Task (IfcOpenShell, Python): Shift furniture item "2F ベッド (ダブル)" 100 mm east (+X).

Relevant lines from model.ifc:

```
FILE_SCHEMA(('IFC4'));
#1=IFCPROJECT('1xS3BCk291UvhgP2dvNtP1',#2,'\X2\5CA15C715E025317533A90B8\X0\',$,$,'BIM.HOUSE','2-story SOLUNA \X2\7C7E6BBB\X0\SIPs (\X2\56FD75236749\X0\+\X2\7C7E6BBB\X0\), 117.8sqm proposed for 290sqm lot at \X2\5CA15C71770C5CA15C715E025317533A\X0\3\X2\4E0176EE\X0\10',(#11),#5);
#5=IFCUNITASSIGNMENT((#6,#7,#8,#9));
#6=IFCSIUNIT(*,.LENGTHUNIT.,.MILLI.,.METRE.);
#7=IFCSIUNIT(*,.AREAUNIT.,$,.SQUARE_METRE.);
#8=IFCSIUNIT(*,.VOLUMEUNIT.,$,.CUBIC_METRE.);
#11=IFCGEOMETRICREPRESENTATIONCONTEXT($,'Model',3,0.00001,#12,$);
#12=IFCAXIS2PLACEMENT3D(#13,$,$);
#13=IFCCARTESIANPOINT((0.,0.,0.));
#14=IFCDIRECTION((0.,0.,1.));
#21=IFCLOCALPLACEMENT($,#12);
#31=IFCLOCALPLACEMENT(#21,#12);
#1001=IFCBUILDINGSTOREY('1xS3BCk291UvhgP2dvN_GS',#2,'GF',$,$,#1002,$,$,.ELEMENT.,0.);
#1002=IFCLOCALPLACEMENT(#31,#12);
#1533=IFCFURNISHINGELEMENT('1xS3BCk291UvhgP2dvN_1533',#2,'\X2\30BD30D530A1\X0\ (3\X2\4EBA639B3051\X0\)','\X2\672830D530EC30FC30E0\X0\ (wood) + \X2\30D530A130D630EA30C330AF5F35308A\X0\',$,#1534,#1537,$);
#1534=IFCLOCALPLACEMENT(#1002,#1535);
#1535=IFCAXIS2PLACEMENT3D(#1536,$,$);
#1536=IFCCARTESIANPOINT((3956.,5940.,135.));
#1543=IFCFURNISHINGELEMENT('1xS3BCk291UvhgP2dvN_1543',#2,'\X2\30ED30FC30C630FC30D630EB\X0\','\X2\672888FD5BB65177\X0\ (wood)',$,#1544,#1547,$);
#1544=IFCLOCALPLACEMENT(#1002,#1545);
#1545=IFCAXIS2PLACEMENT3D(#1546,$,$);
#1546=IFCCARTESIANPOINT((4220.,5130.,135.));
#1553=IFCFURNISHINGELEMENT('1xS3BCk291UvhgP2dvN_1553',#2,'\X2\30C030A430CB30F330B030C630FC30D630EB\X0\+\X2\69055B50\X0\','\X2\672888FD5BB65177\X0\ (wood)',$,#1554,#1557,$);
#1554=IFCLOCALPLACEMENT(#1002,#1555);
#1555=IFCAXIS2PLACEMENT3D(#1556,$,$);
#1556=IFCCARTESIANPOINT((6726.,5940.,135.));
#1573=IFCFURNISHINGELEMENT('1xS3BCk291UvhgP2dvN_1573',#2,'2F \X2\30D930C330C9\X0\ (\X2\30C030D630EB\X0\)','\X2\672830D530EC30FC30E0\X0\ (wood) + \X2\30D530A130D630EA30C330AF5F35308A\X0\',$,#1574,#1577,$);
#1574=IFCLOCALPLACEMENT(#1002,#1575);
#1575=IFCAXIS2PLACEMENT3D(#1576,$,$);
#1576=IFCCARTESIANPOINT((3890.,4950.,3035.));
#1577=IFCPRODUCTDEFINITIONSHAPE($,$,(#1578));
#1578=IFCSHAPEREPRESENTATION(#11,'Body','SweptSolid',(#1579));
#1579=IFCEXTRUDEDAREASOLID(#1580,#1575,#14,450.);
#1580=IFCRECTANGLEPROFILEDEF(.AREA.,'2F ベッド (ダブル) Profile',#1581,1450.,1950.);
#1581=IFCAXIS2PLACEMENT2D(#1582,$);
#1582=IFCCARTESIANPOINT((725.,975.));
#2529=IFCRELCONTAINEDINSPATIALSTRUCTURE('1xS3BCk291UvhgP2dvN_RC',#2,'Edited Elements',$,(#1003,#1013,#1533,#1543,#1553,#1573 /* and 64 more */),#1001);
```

```python
import ifcopenshell
import ifcopenshell.api.geometry
import ifcopenshell.util.placement
import ifcopenshell.util.unit

model = ifcopenshell.open("model.ifc")
unit_scale = ifcopenshell.util.unit.calculate_unit_scale(model)

item = model.by_id(1573)
matrix = ifcopenshell.util.placement.get_local_placement(item.ObjectPlacement)
matrix[0, 3] += 0.1 / unit_scale
ifcopenshell.api.geometry.edit_object_placement(model, product=item, matrix=matrix, is_si=False)

print(ifcopenshell.util.placement.get_local_placement(item.ObjectPlacement).round(3) + 0.0)

model.write("model_v2.ifc")
```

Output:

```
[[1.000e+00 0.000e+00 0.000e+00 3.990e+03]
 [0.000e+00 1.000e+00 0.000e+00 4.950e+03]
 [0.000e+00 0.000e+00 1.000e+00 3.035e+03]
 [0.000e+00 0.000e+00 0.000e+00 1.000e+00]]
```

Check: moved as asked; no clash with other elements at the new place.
